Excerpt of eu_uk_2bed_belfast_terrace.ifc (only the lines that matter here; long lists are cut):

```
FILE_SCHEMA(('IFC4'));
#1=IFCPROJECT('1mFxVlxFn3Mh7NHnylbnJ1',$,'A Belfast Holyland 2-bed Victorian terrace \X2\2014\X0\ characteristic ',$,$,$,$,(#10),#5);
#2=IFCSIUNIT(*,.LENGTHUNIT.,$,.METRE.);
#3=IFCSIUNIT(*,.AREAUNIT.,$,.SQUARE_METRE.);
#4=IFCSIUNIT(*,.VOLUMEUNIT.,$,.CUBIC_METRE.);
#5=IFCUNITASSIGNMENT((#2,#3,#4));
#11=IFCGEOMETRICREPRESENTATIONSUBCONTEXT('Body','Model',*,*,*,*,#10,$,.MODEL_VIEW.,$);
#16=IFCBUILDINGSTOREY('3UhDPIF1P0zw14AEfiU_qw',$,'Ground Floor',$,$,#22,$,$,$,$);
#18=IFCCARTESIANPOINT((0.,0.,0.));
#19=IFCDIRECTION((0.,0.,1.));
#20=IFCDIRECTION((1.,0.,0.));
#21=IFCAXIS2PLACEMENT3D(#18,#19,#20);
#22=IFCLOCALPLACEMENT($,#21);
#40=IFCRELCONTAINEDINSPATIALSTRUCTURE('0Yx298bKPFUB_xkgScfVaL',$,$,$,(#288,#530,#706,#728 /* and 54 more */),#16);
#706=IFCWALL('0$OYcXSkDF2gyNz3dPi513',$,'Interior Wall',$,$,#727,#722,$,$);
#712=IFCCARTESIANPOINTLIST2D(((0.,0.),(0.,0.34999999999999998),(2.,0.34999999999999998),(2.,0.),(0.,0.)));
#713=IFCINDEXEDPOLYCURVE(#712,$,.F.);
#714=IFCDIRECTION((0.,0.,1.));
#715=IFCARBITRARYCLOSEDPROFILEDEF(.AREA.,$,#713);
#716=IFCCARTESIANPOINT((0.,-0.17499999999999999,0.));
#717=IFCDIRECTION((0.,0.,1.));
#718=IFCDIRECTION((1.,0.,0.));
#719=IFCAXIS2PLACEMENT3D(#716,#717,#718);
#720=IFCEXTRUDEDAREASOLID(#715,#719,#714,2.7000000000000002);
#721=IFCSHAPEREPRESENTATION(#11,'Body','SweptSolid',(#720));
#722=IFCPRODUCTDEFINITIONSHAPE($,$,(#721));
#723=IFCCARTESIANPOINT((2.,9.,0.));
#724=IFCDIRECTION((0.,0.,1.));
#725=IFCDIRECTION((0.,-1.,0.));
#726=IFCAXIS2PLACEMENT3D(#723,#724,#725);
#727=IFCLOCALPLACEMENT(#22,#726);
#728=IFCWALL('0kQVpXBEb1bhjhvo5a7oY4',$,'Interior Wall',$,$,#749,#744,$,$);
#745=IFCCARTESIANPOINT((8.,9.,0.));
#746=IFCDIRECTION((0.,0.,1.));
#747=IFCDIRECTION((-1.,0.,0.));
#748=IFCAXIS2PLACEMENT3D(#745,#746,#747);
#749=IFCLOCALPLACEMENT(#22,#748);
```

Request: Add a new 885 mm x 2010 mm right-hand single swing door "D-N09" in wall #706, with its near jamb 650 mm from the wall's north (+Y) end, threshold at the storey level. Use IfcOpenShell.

```python
import numpy as np
import ifcopenshell
import ifcopenshell.api.feature
import ifcopenshell.api.geometry
import ifcopenshell.api.root
import ifcopenshell.api.spatial
import ifcopenshell.geom
import ifcopenshell.util.element
import ifcopenshell.util.placement
import ifcopenshell.util.representation
import ifcopenshell.util.shape
import ifcopenshell.util.unit

model = ifcopenshell.open("eu_uk_2bed_belfast_terrace.ifc")
unit_scale = ifcopenshell.util.unit.calculate_unit_scale(model)
settings = ifcopenshell.geom.settings()


def volume(element):
    """Net volume in cubic metres, openings subtracted."""
    shape = ifcopenshell.geom.create_shape(settings, element)
    return ifcopenshell.util.shape.get_volume(shape.geometry)


wall = model.by_guid("0$OYcXSkDF2gyNz3dPi513")
storey = ifcopenshell.util.element.get_container(wall, ifc_class="IfcBuildingStorey")
context = ifcopenshell.util.representation.get_context(model, "Model", "Body", "MODEL_VIEW")
before = volume(wall)

width, height, from_end, sill = 0.885, 2.01, 0.65, 0.0  # metres

# The wall runs along its own X axis, and the end named is its -X end.
wall_shape = ifcopenshell.geom.create_shape(settings, wall)
x, y, z = ifcopenshell.util.shape.get_vertices(wall_shape.geometry).T
start = x.min() + from_end
face, thickness = float(y.min()), float(y.max() - y.min())
wall_matrix = ifcopenshell.util.placement.get_local_placement(wall.ObjectPlacement)
level = ifcopenshell.util.placement.get_local_placement(storey.ObjectPlacement)[2, 3]


def in_wall(x, y):
    """Placement at x, y metres in the wall's axes, at sill height."""
    matrix = wall_matrix.copy()
    matrix[:, 3] = wall_matrix @ np.array([x / unit_scale, y / unit_scale, 0.0, 1.0])
    matrix[2, 3] = level + sill / unit_scale
    return matrix


# Opening: a box that overshoots both wall faces by 50 mm.
opening = ifcopenshell.api.root.create_entity(model, ifc_class="IfcOpeningElement", predefined_type="OPENING")
box = ifcopenshell.api.geometry.add_wall_representation(
    model, context=context, length=width, height=height, thickness=thickness + 0.1
)
ifcopenshell.api.geometry.assign_representation(model, product=opening, representation=box)
ifcopenshell.api.geometry.edit_object_placement(model, product=opening, matrix=in_wall(start, face - 0.05), is_si=False)
ifcopenshell.api.feature.add_feature(model, feature=opening, element=wall)

door = ifcopenshell.api.root.create_entity(model, ifc_class="IfcDoor", name="D-N09", predefined_type="DOOR")
door.OverallWidth, door.OverallHeight = width / unit_scale, height / unit_scale
door.OperationType = "SINGLE_SWING_RIGHT"
body = ifcopenshell.api.geometry.add_door_representation(
    model,
    context=context,
    overall_width=door.OverallWidth,
    overall_height=door.OverallHeight,
    operation_type="SINGLE_SWING_RIGHT",
    lining_properties={"LiningDepth": thickness / unit_scale, "ThresholdDepth": thickness / unit_scale},
)
ifcopenshell.api.geometry.assign_representation(model, product=door, representation=body)
ifcopenshell.api.spatial.assign_container(model, products=[door], relating_structure=storey)
ifcopenshell.api.feature.add_filling(model, opening=opening, element=door)

# The lining spans the wall, so the door starts at the wall face.
ifcopenshell.api.geometry.edit_object_placement(model, product=door, matrix=in_wall(start, face), is_si=False)

after = volume(wall)

print(f"wall volume {before:.3f} -> {after:.3f} m3")

model.write("eu_uk_2bed_belfast_terrace_edited.ifc")
```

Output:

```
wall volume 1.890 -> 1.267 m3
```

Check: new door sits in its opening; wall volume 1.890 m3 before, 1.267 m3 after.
